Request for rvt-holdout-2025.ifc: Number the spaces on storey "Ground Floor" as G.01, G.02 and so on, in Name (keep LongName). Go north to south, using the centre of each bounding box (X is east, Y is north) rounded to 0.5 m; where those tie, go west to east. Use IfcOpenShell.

First a look at what the model holds.

```python
import ifcopenshell
import ifcopenshell.util.element
import ifcopenshell.util.placement

model = ifcopenshell.open("rvt-holdout-2025.ifc")
print(model.schema)
storey = next(s for s in model.by_type("IfcBuildingStorey") if s.Name == "Ground Floor")
spaces = [e for e in ifcopenshell.util.element.get_decomposition(storey) if e.is_a("IfcSpace")]
for e in sorted(spaces, key=lambda e: e.id()):
    origin = ifcopenshell.util.placement.get_local_placement(e.ObjectPlacement)[:3, 3]
    print(e.id(), e.Name, e.LongName, origin.round(2) + 0.0, sep=" | ")
```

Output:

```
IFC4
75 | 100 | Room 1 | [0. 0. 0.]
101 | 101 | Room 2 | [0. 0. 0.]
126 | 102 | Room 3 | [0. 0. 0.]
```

```python
import ifcopenshell
import ifcopenshell.geom
import ifcopenshell.util.element
import ifcopenshell.util.shape

model = ifcopenshell.open("rvt-holdout-2025.ifc")
settings = ifcopenshell.geom.settings()
settings.set("use-world-coords", True)


def centre(element):
    shape = ifcopenshell.geom.create_shape(settings, element)
    return ifcopenshell.util.shape.get_bbox_centroid(shape.geometry)


storey = next(s for s in model.by_type("IfcBuildingStorey") if s.Name == "Ground Floor")
spaces = [e for e in ifcopenshell.util.element.get_decomposition(storey) if e.is_a("IfcSpace")]

# Insertion points can sit at a corner or the storey origin, so sort by the geometry (in metres).
centres = {e: centre(e) for e in spaces}
spaces.sort(key=lambda e: (-round(centres[e][1] / 0.5), centres[e][0]))

for i, e in enumerate(spaces, start=1):
    number = f"G.{i:02d}"
    e.Name = number
    print(e.id(), number)

model.write("rvt-holdout-2025_rev.ifc")
```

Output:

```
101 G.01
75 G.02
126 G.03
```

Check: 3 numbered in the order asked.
